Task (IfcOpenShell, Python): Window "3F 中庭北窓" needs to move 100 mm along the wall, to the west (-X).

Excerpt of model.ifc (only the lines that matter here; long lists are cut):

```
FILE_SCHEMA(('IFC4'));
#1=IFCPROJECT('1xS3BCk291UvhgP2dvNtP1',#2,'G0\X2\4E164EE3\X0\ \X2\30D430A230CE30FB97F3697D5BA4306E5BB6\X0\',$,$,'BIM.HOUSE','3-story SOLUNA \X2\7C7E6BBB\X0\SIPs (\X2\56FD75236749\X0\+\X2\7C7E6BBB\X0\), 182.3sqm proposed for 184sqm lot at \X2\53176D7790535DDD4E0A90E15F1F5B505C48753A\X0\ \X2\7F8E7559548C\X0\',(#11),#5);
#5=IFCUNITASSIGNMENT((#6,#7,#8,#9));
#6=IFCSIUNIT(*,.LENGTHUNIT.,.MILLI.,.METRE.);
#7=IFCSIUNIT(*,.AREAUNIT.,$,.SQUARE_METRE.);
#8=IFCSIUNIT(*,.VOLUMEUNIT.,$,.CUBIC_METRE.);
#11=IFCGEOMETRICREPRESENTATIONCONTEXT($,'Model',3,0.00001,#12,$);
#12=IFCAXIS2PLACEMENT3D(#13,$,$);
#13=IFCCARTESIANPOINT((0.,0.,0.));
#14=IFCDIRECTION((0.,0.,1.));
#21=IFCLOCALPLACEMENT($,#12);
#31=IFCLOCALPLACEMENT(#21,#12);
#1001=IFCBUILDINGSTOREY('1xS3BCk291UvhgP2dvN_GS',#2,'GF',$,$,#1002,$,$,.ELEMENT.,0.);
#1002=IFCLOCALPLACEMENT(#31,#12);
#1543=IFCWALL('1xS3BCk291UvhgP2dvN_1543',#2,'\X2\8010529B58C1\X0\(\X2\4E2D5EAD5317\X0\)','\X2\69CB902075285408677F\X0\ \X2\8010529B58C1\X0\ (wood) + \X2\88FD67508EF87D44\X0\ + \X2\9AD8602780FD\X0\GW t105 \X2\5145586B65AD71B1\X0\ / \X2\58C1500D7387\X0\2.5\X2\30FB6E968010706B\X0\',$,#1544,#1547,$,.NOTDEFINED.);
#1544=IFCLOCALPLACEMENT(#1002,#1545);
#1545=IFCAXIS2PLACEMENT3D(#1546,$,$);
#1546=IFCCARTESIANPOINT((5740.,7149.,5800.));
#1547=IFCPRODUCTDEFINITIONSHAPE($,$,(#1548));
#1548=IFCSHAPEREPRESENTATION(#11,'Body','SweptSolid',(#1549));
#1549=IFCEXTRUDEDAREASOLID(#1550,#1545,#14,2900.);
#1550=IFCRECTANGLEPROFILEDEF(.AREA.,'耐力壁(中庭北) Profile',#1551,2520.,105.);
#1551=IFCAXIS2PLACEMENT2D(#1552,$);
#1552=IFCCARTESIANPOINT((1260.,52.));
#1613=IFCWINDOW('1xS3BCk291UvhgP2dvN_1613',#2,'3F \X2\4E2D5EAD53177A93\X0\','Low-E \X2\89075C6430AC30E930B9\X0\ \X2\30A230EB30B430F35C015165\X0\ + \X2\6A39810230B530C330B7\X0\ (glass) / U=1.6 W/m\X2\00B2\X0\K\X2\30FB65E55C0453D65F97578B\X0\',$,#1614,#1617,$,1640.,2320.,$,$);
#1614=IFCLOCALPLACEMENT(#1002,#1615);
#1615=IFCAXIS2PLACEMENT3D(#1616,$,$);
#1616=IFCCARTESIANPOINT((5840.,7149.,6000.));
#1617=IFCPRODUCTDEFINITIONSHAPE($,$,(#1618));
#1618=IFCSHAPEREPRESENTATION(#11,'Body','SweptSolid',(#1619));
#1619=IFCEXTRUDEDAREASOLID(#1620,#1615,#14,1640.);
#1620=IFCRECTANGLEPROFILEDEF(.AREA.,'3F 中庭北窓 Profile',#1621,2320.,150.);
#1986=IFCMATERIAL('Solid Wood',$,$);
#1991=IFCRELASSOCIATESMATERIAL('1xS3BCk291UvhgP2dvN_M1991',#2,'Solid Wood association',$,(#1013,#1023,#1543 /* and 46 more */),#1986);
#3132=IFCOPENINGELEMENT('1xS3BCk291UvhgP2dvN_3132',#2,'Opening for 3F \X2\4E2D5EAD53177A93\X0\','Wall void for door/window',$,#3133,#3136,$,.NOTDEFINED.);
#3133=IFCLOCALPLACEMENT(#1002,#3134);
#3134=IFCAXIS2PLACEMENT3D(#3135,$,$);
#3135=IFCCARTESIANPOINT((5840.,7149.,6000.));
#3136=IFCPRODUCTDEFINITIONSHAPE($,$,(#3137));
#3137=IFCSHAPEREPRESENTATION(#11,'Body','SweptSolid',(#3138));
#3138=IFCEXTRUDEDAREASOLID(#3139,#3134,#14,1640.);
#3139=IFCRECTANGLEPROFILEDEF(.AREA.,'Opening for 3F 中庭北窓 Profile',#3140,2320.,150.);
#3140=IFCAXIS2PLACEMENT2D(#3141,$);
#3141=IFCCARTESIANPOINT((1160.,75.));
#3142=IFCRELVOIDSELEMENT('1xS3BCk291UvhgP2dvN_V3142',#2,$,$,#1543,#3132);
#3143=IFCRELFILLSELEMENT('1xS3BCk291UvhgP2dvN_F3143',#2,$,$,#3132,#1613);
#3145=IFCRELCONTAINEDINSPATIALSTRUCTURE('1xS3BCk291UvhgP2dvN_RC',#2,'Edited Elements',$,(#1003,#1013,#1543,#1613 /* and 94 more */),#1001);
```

```python
import ifcopenshell
import ifcopenshell.api.geometry
import ifcopenshell.util.placement
import ifcopenshell.util.unit

model = ifcopenshell.open("model.ifc")
unit_scale = ifcopenshell.util.unit.calculate_unit_scale(model)

window = model.by_guid("1xS3BCk291UvhgP2dvN_1613")
opening = window.FillsVoids[0].RelatingOpeningElement
wall = opening.VoidsElements[0].RelatingBuildingElement

wall_matrix = ifcopenshell.util.placement.get_local_placement(wall.ObjectPlacement)
shift = wall_matrix[:3, 0] * -0.1 / unit_scale
before = ifcopenshell.util.placement.get_local_placement(window.ObjectPlacement)[:3, 3].copy()

# The window is not placed relative to its opening, so move both.
for product in (opening, window):
    matrix = ifcopenshell.util.placement.get_local_placement(product.ObjectPlacement)
    matrix[:3, 3] += shift
    ifcopenshell.api.geometry.edit_object_placement(model, product=product, matrix=matrix, is_si=False)

after = ifcopenshell.util.placement.get_local_placement(window.ObjectPlacement)[:3, 3]
print("window moved by", (after - before).round(3) + 0.0)

model.write("model-out.ifc")
```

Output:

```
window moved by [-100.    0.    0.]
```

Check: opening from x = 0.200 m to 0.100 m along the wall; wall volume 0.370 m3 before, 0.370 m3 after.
